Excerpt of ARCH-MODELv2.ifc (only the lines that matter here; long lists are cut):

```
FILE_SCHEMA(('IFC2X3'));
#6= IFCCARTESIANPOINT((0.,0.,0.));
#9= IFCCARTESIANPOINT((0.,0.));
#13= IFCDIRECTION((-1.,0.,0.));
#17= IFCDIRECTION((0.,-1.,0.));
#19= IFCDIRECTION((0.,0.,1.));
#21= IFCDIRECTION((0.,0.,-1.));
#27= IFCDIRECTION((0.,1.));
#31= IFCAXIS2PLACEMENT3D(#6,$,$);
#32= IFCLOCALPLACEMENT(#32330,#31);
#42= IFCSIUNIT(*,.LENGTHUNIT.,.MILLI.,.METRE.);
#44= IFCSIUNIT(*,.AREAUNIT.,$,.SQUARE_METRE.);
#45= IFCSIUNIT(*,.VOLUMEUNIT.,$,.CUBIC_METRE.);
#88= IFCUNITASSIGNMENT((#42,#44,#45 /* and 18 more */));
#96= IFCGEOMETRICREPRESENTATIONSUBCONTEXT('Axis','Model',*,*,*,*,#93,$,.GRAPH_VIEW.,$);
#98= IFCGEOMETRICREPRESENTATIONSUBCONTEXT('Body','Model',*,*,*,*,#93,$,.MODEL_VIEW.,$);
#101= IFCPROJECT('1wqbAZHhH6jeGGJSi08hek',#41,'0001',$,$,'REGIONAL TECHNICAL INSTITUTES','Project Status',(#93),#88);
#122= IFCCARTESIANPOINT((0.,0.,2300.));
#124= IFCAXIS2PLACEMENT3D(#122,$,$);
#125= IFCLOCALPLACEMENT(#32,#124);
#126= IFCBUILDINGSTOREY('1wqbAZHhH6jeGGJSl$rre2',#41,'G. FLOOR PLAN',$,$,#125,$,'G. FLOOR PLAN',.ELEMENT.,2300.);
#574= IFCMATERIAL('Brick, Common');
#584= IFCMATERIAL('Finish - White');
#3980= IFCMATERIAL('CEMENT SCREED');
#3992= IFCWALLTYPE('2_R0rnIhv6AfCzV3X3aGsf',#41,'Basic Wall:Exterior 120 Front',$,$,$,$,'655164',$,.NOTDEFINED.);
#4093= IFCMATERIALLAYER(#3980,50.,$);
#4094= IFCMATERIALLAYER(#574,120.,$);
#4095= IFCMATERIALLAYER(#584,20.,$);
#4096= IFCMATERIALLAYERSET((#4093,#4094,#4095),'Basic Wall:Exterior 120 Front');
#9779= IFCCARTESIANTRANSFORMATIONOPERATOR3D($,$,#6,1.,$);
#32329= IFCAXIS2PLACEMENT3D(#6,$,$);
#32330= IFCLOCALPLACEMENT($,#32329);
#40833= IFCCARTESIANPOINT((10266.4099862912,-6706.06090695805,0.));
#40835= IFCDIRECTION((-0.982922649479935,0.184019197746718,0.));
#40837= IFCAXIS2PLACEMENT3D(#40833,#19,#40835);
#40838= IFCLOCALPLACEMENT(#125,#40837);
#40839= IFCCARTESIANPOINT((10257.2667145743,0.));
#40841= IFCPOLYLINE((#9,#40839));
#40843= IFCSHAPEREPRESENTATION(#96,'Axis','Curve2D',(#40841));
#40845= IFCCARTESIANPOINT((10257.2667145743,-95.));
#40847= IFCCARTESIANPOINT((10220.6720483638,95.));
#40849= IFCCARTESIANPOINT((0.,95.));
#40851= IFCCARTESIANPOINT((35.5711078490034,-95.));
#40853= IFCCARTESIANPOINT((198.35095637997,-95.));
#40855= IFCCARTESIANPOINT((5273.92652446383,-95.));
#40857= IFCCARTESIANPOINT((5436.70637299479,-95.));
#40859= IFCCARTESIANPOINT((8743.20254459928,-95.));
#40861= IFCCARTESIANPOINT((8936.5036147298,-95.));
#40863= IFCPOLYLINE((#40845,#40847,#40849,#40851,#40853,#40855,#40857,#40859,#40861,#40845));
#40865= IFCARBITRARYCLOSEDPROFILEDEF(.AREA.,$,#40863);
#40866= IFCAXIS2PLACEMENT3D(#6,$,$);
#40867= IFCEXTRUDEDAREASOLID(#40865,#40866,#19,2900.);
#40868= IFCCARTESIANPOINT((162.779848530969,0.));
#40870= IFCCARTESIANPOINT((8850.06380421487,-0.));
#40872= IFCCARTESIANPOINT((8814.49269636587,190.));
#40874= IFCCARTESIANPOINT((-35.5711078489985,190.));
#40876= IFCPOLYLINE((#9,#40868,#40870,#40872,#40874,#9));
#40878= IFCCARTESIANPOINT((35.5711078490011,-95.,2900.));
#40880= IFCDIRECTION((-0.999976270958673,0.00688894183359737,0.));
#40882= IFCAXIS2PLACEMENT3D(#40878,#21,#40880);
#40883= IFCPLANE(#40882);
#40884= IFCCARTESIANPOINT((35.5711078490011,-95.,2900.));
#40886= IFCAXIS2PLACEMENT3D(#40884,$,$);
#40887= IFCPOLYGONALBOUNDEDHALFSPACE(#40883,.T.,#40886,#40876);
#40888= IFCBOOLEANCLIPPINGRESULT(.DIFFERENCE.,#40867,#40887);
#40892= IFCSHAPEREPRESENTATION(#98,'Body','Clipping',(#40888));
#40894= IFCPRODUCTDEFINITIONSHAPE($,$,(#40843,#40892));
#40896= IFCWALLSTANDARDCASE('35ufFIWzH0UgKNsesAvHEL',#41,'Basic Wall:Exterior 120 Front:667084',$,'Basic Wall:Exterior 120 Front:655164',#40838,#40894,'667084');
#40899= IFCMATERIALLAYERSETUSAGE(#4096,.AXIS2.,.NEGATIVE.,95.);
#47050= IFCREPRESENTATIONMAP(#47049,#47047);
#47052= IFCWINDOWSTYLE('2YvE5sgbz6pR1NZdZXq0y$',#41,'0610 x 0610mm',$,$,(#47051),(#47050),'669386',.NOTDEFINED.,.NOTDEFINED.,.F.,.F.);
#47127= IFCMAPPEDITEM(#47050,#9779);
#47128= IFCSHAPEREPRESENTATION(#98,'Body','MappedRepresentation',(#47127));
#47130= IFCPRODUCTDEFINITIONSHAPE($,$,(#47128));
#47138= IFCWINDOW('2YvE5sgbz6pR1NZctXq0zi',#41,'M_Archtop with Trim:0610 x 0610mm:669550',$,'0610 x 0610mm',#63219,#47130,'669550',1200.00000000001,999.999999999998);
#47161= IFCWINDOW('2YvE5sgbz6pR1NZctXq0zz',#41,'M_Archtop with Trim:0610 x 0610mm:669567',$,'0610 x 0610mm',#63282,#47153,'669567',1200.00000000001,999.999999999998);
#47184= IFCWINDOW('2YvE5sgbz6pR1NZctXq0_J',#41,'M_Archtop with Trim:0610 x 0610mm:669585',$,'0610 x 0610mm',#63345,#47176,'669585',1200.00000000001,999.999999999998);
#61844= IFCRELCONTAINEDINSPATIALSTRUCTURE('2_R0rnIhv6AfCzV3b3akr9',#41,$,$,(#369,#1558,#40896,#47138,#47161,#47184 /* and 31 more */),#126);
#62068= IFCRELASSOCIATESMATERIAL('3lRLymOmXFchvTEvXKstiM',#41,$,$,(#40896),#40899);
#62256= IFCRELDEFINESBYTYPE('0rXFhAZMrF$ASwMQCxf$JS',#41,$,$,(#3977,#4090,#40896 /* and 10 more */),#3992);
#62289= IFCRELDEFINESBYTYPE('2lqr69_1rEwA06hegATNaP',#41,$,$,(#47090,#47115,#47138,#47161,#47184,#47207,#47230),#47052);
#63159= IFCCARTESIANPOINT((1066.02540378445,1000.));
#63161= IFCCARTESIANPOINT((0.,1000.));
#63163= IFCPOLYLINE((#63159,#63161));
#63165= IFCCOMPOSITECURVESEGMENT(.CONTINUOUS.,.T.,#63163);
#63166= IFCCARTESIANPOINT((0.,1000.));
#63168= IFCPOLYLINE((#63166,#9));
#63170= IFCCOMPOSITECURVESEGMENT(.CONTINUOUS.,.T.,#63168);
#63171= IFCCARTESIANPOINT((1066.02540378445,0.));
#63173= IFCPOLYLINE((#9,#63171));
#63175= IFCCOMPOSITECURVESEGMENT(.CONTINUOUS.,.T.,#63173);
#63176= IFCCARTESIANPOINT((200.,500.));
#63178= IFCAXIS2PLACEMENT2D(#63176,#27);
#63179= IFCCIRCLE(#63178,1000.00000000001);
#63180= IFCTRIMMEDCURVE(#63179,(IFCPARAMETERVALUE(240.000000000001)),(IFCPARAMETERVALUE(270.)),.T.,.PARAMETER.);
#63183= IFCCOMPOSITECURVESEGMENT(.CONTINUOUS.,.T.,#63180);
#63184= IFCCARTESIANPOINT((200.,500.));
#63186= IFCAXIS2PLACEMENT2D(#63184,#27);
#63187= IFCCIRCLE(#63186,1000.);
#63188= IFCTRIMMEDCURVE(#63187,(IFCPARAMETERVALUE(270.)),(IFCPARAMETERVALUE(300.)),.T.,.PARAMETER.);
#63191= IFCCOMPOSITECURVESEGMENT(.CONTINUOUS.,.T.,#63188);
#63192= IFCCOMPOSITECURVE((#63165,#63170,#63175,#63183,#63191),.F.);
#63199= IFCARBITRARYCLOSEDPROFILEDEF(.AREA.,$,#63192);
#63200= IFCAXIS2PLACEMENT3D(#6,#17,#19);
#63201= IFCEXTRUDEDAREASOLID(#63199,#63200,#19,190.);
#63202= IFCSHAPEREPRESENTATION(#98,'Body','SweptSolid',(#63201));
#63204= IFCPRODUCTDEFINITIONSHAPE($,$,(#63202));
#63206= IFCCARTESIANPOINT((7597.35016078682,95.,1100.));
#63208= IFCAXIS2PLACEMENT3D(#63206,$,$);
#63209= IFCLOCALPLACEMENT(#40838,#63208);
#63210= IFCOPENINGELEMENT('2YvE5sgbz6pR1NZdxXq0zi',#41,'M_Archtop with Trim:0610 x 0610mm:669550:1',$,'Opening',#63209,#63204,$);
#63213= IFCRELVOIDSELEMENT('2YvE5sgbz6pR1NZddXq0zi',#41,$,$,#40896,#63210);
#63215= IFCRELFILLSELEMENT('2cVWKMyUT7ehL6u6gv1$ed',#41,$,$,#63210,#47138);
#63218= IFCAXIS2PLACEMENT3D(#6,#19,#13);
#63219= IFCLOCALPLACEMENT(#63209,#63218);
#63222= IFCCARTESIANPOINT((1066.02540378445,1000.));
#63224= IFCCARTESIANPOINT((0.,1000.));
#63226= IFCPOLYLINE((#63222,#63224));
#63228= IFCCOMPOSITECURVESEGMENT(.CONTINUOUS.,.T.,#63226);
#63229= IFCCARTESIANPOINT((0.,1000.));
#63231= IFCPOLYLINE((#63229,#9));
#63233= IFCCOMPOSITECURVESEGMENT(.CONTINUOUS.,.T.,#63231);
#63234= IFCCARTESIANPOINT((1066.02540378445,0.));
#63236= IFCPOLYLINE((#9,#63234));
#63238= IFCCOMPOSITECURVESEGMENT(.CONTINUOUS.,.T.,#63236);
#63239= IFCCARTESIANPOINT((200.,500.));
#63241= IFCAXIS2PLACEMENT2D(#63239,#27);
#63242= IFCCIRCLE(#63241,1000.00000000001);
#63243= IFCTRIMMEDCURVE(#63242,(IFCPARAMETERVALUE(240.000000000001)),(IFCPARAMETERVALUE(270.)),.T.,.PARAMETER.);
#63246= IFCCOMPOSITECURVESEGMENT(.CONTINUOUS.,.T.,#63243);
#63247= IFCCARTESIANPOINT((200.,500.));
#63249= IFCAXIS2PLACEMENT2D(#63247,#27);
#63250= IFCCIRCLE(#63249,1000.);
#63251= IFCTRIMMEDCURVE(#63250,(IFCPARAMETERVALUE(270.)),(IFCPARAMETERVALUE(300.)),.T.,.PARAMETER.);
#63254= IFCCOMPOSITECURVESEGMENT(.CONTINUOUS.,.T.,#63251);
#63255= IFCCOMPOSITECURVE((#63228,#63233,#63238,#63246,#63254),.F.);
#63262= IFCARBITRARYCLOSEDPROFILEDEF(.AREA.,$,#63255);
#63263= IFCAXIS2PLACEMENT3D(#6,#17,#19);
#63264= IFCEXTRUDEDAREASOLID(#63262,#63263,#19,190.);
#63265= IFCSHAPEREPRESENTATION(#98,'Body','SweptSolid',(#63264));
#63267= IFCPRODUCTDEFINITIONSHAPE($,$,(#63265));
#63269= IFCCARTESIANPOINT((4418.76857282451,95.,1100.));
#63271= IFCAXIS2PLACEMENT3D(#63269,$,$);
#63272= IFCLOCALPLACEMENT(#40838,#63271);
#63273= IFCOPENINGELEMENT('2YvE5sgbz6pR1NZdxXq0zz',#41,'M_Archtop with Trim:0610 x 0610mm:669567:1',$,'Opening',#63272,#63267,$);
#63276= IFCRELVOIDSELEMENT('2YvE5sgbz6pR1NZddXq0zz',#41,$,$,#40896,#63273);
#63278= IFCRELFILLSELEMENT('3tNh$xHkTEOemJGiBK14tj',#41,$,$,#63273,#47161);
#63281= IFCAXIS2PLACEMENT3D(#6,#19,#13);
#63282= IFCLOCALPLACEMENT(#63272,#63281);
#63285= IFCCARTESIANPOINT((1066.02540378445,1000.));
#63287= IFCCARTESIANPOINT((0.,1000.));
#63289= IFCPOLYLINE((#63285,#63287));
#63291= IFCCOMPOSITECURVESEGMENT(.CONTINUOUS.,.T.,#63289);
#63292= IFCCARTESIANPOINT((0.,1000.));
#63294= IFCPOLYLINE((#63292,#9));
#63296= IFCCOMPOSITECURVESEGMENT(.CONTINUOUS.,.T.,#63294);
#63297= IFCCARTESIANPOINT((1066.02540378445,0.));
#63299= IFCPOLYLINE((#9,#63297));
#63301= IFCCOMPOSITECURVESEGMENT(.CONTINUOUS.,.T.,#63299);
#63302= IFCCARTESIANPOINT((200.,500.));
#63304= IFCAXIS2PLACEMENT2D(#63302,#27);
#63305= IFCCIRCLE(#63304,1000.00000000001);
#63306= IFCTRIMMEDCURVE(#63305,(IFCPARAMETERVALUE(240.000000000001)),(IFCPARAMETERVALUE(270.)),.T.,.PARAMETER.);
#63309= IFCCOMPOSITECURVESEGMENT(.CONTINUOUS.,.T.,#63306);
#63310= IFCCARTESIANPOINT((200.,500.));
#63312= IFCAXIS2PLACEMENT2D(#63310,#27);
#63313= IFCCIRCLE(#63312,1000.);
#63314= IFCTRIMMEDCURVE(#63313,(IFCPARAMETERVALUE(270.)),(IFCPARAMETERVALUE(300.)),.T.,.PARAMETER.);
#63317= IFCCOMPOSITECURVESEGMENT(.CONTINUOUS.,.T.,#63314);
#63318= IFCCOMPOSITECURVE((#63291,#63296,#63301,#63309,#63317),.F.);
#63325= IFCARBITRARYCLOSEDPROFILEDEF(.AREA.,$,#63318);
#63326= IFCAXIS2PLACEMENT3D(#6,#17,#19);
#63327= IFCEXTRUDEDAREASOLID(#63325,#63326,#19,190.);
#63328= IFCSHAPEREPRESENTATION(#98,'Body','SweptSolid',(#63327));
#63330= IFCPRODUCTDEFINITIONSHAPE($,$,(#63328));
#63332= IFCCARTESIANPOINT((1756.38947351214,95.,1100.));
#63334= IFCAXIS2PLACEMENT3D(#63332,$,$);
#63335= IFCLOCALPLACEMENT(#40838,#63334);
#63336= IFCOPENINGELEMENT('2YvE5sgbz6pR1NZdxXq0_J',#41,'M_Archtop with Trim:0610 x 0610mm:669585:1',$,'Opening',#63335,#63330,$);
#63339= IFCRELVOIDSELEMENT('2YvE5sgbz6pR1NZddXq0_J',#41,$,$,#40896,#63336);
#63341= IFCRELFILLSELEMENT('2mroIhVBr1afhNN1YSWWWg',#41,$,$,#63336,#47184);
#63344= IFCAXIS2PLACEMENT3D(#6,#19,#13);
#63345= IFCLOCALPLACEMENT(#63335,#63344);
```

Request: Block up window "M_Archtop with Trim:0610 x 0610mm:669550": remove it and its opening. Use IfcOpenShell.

```python
import ifcopenshell
import ifcopenshell.api.feature
import ifcopenshell.api.root
import ifcopenshell.geom
import ifcopenshell.util.shape

model = ifcopenshell.open("ARCH-MODELv2.ifc")
settings = ifcopenshell.geom.settings()


def volume(element):
    """Net volume in cubic metres, openings subtracted."""
    shape = ifcopenshell.geom.create_shape(settings, element)
    return ifcopenshell.util.shape.get_volume(shape.geometry)


window = model.by_id(47138)
opening = window.FillsVoids[0].RelatingOpeningElement
wall = opening.VoidsElements[0].RelatingBuildingElement
before = volume(wall)

ifcopenshell.api.root.remove_product(model, product=window)
ifcopenshell.api.feature.remove_feature(model, feature=opening)

after = volume(wall)

print(f"wall volume {before:.3f} -> {after:.3f} m3")

model.write("ARCH-MODELv2_updated.ifc")
```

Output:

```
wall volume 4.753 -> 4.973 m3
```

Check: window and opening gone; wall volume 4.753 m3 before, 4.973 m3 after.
